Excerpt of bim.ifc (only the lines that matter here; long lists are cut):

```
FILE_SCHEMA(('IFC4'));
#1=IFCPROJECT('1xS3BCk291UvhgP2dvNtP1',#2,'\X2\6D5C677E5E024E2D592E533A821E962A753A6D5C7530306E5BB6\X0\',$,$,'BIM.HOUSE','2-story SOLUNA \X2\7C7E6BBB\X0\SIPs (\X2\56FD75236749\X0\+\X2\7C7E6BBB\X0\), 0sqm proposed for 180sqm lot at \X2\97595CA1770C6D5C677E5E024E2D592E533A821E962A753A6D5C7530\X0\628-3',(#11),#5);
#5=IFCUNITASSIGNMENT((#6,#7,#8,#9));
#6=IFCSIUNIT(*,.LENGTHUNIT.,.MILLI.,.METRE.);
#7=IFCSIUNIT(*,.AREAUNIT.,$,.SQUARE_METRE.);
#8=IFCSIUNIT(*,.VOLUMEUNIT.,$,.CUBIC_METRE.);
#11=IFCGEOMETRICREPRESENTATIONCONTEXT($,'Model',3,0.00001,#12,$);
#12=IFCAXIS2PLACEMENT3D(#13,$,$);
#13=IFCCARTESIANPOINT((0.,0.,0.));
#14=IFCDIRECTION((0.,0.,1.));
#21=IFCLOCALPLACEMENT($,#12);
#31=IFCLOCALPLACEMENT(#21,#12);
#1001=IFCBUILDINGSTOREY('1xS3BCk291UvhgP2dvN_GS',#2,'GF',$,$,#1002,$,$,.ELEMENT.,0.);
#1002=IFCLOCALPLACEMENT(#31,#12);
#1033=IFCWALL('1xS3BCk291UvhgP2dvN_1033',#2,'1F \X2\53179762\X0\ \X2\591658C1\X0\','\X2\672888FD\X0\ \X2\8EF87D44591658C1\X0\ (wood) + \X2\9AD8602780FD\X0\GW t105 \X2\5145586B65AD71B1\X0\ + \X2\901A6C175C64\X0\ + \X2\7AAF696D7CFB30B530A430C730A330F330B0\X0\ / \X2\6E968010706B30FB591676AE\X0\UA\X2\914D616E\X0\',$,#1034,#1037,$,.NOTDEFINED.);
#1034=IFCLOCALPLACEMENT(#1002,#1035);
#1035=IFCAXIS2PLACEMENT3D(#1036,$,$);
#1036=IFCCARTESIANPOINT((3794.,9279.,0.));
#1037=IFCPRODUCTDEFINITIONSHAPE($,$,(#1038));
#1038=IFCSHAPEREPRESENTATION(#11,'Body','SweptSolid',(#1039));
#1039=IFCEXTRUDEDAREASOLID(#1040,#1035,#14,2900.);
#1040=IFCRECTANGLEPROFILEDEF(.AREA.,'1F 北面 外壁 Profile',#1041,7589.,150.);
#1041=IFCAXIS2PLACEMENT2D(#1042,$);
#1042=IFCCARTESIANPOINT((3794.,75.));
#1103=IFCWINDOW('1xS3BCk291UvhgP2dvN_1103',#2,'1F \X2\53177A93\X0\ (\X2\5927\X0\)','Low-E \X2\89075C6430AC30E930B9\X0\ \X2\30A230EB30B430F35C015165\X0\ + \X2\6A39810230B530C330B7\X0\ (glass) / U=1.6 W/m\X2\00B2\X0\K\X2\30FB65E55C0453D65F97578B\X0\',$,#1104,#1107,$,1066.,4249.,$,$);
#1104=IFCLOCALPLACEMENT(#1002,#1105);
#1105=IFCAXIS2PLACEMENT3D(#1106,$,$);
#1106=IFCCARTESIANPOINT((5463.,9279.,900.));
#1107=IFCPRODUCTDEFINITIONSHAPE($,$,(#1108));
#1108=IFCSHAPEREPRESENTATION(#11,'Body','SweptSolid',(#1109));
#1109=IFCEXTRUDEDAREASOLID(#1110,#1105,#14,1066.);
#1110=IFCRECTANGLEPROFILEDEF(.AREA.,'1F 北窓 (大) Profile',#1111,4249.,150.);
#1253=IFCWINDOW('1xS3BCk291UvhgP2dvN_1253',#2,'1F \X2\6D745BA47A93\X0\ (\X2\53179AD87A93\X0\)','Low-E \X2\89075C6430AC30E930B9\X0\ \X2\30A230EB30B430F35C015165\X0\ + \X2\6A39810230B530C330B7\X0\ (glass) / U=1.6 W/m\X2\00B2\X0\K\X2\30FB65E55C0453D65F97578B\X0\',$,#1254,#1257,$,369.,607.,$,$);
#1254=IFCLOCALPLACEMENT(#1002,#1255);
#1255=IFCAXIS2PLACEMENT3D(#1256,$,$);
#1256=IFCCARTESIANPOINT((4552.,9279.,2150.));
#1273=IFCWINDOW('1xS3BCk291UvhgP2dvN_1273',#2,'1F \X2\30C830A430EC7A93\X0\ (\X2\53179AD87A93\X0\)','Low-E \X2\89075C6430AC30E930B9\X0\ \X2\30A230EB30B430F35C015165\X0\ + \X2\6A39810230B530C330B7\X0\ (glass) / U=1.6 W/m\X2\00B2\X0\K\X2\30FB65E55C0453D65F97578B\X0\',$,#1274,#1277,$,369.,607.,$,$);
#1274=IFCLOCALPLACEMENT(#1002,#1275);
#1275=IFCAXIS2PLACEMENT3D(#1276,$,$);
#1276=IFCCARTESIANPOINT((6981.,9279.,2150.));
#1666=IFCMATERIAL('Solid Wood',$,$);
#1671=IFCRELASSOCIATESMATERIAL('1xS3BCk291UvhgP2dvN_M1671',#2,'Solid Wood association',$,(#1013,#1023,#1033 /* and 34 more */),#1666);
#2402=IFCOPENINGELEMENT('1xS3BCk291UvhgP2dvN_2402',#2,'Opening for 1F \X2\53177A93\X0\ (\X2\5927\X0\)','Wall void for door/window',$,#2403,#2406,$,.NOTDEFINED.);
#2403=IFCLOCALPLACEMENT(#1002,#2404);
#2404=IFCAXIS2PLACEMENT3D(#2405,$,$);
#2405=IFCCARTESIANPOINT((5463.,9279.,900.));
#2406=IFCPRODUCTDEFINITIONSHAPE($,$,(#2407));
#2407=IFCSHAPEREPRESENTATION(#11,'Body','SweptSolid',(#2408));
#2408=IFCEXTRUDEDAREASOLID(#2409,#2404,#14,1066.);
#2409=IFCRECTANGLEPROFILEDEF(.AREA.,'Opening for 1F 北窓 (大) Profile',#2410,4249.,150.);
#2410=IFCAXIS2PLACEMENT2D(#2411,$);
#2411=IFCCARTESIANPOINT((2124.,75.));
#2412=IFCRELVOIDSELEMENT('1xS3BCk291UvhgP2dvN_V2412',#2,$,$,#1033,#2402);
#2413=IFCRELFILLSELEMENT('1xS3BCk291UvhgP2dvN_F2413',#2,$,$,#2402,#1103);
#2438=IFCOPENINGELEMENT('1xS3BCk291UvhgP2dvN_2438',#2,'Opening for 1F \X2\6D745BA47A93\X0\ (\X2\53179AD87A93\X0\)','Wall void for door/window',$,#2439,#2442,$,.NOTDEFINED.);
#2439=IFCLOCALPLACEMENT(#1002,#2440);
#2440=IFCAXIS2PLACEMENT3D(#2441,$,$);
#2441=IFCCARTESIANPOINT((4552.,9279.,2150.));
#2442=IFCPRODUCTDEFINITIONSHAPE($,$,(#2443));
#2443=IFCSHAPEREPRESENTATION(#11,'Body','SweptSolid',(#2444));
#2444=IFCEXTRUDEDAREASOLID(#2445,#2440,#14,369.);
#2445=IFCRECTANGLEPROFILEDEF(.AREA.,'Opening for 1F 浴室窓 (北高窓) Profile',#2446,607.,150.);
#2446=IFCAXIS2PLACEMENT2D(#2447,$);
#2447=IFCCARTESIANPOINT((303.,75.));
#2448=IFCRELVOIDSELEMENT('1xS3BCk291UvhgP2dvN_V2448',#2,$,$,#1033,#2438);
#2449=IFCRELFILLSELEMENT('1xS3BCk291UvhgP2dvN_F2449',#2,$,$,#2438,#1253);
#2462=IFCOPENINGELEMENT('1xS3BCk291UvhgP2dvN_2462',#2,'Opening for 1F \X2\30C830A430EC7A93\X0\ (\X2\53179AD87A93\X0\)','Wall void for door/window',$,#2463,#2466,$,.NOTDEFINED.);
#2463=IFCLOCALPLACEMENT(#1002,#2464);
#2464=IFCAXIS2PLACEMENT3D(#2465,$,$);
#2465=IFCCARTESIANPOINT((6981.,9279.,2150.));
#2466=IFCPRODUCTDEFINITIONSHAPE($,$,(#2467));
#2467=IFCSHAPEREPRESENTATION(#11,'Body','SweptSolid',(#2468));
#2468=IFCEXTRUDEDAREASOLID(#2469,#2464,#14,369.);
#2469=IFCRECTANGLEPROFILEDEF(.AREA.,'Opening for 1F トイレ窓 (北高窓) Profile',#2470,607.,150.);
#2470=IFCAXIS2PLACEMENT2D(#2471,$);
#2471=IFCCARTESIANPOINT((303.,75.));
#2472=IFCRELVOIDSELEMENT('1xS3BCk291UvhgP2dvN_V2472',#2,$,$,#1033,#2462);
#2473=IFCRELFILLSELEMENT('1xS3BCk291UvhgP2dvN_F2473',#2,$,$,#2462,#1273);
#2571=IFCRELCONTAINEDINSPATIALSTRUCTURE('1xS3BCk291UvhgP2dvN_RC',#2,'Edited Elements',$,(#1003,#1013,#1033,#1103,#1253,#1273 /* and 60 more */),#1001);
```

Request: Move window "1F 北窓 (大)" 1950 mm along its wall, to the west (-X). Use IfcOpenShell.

```python
import ifcopenshell
import ifcopenshell.api.geometry
import ifcopenshell.util.placement

model = ifcopenshell.open("bim.ifc")

window = model.by_guid("1xS3BCk291UvhgP2dvN_1103")
opening = window.FillsVoids[0].RelatingOpeningElement
wall = opening.VoidsElements[0].RelatingBuildingElement

wall_matrix = ifcopenshell.util.placement.get_local_placement(wall.ObjectPlacement)
shift = wall_matrix[:3, 0] * -1950.0
before = ifcopenshell.util.placement.get_local_placement(window.ObjectPlacement)[:3, 3].copy()

# The window is not placed relative to its opening, so move both.
for product in (opening, window):
    matrix = ifcopenshell.util.placement.get_local_placement(product.ObjectPlacement)
    matrix[:3, 3] += shift
    ifcopenshell.api.geometry.edit_object_placement(model, product=product, matrix=matrix, is_si=False)

after = ifcopenshell.util.placement.get_local_placement(window.ObjectPlacement)[:3, 3]
print("window moved by", (after - before).round(3) + 0.0)

model.write("bim_edited.ifc")
```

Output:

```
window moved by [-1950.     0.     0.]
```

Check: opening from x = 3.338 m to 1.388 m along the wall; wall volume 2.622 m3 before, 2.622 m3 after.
